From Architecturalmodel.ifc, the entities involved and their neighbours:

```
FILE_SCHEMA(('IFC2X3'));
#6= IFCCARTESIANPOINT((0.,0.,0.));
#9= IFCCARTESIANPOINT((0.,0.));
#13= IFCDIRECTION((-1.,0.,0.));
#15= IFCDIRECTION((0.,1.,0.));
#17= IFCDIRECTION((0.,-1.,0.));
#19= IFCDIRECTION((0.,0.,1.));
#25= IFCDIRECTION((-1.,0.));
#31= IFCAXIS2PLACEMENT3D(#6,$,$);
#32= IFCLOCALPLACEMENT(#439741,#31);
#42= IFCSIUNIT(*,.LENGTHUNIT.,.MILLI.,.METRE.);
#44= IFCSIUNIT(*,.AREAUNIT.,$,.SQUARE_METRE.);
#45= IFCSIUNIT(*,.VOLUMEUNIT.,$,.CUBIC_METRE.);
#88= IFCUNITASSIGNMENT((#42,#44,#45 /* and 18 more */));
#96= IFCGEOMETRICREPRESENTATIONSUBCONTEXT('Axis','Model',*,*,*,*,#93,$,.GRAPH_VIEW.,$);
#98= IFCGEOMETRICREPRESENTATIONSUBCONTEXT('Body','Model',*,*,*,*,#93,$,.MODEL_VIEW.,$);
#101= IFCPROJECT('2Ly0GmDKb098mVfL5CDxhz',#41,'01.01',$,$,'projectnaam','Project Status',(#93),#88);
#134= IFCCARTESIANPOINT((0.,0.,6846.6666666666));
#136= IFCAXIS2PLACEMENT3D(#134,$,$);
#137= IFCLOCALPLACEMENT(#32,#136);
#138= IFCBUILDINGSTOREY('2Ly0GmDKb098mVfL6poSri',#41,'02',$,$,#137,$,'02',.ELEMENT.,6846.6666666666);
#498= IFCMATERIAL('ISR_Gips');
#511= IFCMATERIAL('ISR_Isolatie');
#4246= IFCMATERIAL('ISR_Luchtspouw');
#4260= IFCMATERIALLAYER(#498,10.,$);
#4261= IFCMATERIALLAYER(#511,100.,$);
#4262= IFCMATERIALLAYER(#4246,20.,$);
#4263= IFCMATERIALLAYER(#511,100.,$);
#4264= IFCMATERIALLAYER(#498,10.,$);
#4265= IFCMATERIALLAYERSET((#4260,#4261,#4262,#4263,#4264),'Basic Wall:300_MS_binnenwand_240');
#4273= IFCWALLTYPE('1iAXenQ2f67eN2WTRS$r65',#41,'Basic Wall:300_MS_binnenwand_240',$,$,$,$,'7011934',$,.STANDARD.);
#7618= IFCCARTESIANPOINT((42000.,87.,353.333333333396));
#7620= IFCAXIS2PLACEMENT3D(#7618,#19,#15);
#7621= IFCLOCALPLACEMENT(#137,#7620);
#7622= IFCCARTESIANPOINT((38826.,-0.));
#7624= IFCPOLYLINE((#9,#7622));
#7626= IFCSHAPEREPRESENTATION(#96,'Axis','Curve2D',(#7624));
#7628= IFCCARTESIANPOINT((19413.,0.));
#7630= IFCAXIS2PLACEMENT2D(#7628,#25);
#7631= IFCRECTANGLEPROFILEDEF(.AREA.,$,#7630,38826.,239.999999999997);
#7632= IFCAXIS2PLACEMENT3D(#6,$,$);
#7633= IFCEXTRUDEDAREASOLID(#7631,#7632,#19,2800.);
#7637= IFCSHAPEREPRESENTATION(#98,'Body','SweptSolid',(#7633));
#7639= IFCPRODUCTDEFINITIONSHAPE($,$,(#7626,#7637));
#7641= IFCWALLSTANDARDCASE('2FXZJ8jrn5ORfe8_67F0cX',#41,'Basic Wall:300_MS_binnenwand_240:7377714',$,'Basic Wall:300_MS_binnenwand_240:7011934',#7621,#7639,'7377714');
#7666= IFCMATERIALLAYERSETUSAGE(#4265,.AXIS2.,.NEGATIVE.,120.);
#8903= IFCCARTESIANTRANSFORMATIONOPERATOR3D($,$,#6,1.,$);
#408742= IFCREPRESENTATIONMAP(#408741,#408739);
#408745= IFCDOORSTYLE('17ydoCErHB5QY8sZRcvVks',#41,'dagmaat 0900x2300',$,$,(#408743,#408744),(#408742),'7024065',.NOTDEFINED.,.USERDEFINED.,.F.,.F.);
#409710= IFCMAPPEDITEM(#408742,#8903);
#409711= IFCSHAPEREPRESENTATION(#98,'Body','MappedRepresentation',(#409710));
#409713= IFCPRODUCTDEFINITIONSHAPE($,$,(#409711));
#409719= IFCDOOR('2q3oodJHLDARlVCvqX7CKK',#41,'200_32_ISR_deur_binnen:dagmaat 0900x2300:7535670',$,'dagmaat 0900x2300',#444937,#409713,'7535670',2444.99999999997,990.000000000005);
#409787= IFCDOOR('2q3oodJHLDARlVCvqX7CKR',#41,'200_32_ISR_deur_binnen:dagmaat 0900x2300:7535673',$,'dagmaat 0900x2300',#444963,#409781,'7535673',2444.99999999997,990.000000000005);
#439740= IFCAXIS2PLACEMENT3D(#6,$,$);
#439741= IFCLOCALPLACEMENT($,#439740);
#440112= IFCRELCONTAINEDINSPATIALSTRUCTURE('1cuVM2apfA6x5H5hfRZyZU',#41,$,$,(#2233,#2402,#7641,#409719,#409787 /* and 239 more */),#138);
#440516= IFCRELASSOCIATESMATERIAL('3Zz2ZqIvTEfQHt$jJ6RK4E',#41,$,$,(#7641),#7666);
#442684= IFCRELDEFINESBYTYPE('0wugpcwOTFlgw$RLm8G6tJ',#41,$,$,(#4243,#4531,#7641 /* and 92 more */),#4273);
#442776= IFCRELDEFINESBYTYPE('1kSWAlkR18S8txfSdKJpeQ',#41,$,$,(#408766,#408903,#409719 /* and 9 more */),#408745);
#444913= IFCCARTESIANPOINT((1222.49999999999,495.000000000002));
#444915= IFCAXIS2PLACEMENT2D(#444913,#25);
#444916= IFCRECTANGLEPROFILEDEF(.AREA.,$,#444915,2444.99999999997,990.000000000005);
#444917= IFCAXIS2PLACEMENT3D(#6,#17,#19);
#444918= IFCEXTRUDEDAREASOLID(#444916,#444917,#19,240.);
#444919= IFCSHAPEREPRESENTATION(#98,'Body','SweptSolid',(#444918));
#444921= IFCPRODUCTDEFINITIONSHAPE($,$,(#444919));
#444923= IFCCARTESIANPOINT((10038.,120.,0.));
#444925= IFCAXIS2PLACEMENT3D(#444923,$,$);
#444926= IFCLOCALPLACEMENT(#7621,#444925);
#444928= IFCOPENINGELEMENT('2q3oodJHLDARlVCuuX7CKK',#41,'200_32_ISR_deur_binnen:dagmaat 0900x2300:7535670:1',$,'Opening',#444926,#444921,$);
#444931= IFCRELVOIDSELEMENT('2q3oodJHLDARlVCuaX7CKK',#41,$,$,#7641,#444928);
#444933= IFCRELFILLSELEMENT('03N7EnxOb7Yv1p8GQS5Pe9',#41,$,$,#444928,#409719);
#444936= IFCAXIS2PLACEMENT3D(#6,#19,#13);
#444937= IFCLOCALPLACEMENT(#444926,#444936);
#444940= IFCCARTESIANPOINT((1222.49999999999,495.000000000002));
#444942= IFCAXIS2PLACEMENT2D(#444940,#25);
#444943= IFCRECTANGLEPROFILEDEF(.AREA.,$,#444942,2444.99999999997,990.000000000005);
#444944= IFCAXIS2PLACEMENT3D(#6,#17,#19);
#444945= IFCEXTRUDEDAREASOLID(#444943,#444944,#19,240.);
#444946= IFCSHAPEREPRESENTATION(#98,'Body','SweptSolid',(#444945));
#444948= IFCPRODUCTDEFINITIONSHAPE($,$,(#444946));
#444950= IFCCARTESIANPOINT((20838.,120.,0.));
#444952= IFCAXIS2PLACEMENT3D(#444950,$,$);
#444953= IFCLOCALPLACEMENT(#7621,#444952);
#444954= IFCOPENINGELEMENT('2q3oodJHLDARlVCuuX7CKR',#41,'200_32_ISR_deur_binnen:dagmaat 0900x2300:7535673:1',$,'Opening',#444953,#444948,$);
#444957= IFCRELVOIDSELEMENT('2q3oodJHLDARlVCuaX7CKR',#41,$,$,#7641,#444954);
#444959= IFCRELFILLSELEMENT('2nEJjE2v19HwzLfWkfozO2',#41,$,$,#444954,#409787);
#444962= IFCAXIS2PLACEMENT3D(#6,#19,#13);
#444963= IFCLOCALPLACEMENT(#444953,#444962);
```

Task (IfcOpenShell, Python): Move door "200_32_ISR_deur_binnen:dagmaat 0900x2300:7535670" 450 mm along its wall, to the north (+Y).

```python
import ifcopenshell
import ifcopenshell.api.geometry
import ifcopenshell.util.placement
import ifcopenshell.util.unit

model = ifcopenshell.open("Architecturalmodel.ifc")
unit_scale = ifcopenshell.util.unit.calculate_unit_scale(model)

door = model.by_guid("2q3oodJHLDARlVCvqX7CKK")
opening = door.FillsVoids[0].RelatingOpeningElement
wall = opening.VoidsElements[0].RelatingBuildingElement

wall_matrix = ifcopenshell.util.placement.get_local_placement(wall.ObjectPlacement)
shift = wall_matrix[:3, 0] * 0.45 / unit_scale
before = ifcopenshell.util.placement.get_local_placement(door.ObjectPlacement)[:3, 3].copy()

# The door is placed relative to its opening, so it follows when the opening moves.
matrix = ifcopenshell.util.placement.get_local_placement(opening.ObjectPlacement)
matrix[:3, 3] += shift
ifcopenshell.api.geometry.edit_object_placement(
    model, product=opening, matrix=matrix, is_si=False, should_transform_children=True
)

after = ifcopenshell.util.placement.get_local_placement(door.ObjectPlacement)[:3, 3]
print("door moved by", (after - before).round(3) + 0.0)

model.write("Architecturalmodel-out.ifc")
```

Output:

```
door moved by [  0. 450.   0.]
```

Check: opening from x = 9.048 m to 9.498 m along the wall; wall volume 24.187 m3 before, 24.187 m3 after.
